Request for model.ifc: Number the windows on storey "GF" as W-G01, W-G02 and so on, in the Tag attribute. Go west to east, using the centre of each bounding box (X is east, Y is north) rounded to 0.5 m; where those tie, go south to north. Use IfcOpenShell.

First a look at what the model holds.

```python
import ifcopenshell
import ifcopenshell.util.element
import ifcopenshell.util.placement

model = ifcopenshell.open("model.ifc")
print(model.schema)
storey = next(s for s in model.by_type("IfcBuildingStorey") if s.Name == "GF")
windows = [e for e in ifcopenshell.util.element.get_decomposition(storey) if e.is_a("IfcWindow")]
for e in sorted(windows, key=lambda e: e.id()):
    origin = ifcopenshell.util.placement.get_local_placement(e.ObjectPlacement)[:3, 3]
    print(e.id(), e.Tag, e.Name, origin.round(2) + 0.0, sep=" | ")
```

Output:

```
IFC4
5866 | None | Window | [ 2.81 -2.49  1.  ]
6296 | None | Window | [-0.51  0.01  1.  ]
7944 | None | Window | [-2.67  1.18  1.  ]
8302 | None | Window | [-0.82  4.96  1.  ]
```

```python
import ifcopenshell
import ifcopenshell.geom
import ifcopenshell.util.element
import ifcopenshell.util.shape

model = ifcopenshell.open("model.ifc")
settings = ifcopenshell.geom.settings()
settings.set("use-world-coords", True)


def centre(element):
    shape = ifcopenshell.geom.create_shape(settings, element)
    return ifcopenshell.util.shape.get_bbox_centroid(shape.geometry)


storey = next(s for s in model.by_type("IfcBuildingStorey") if s.Name == "GF")
windows = [e for e in ifcopenshell.util.element.get_decomposition(storey) if e.is_a("IfcWindow")]

# Insertion points can sit at a corner or the storey origin, so sort by the geometry (in metres).
centres = {e: centre(e) for e in windows}
windows.sort(key=lambda e: (round(centres[e][0] / 0.5), centres[e][1]))

for i, e in enumerate(windows, start=1):
    number = f"W-G{i:02d}"
    e.Tag = number
    print(e.id(), number)

model.write("model_updated.ifc")
```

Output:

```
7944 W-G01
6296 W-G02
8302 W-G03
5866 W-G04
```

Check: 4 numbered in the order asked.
